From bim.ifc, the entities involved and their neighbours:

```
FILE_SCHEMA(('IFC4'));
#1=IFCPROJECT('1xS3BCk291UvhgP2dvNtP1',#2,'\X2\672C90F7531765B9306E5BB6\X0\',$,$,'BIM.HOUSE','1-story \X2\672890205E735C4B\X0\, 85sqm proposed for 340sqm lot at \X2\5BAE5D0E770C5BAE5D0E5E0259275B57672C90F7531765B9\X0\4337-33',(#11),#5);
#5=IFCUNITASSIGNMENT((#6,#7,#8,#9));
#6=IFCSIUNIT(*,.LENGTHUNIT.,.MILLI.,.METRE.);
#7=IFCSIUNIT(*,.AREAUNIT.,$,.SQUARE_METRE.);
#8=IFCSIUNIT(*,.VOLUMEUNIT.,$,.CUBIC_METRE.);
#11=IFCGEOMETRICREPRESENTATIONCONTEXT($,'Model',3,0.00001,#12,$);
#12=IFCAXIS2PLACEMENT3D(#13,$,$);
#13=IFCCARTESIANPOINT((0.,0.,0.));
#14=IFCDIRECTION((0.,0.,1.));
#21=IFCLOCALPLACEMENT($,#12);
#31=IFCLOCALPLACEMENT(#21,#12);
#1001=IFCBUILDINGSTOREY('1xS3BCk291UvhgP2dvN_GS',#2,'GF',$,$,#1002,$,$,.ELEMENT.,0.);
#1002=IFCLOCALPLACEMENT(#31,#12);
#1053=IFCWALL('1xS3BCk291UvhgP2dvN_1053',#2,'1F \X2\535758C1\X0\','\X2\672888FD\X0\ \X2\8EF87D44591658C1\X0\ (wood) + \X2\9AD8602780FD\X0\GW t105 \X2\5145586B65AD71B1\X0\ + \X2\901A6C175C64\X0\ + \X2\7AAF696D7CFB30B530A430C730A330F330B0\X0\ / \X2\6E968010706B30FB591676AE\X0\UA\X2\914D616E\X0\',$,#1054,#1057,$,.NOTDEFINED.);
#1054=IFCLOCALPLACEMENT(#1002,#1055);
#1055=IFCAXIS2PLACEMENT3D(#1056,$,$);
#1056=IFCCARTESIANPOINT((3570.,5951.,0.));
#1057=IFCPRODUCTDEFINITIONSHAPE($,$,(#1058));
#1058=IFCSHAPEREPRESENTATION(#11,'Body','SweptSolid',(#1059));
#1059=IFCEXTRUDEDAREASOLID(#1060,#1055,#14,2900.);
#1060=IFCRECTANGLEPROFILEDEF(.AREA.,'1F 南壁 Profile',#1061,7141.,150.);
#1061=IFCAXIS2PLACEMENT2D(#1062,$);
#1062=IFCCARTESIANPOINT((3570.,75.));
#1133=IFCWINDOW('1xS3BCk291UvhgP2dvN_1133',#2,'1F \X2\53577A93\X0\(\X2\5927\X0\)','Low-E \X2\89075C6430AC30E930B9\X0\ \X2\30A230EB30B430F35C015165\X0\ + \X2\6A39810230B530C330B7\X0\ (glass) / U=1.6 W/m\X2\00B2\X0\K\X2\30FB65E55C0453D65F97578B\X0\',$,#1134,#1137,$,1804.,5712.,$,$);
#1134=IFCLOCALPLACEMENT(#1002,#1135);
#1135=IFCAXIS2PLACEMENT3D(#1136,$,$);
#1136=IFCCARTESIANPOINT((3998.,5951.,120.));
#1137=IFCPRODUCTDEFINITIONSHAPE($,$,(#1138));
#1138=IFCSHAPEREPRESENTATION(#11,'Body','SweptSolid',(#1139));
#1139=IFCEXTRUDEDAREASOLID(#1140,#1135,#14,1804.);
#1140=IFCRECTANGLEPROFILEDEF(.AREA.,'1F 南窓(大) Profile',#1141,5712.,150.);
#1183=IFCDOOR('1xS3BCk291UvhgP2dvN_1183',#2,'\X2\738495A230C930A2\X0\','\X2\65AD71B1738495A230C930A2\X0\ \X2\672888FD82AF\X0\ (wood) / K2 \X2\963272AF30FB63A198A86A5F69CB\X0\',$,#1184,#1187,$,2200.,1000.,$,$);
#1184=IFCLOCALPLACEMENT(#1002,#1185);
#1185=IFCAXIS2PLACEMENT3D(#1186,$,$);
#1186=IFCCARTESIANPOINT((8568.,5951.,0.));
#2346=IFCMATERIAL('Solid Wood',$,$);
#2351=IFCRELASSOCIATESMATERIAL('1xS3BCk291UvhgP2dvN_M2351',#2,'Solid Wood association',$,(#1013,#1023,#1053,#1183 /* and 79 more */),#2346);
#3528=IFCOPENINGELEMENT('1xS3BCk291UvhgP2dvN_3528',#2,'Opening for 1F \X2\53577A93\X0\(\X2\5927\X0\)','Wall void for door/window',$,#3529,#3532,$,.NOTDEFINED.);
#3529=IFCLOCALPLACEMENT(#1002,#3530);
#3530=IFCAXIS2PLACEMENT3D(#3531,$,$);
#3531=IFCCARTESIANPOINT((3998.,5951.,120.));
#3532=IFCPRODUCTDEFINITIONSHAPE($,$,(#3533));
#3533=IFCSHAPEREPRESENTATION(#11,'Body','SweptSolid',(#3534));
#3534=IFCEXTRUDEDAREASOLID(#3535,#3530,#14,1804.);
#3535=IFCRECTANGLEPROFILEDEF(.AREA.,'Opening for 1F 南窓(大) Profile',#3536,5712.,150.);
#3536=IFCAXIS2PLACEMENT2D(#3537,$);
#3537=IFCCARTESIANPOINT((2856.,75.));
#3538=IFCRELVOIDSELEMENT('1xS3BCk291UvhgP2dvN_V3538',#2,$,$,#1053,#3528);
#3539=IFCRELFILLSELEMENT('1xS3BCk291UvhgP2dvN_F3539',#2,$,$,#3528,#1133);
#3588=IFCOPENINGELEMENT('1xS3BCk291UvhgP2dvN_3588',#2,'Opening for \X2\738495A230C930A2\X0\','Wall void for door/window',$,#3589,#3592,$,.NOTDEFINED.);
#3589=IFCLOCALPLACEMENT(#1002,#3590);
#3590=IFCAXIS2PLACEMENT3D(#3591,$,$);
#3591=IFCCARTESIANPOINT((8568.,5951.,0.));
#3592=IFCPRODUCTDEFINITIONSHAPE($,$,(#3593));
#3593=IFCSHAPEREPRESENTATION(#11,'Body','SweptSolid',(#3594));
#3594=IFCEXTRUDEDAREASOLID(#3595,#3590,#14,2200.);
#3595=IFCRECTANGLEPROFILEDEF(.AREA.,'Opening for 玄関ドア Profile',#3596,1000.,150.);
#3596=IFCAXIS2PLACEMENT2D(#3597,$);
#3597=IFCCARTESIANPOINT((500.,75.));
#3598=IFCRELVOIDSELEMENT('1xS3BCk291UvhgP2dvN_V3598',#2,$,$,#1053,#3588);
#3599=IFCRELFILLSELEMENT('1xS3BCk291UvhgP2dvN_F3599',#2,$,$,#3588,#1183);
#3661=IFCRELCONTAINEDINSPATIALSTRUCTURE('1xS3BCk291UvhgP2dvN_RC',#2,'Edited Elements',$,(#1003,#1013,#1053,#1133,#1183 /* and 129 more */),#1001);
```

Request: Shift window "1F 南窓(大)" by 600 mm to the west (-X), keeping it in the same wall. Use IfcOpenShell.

```python
import ifcopenshell
import ifcopenshell.api.geometry
import ifcopenshell.util.placement

model = ifcopenshell.open("bim.ifc")

window = model.by_guid("1xS3BCk291UvhgP2dvN_1133")
opening = window.FillsVoids[0].RelatingOpeningElement
wall = opening.VoidsElements[0].RelatingBuildingElement

wall_matrix = ifcopenshell.util.placement.get_local_placement(wall.ObjectPlacement)
shift = wall_matrix[:3, 0] * -600.0
before = ifcopenshell.util.placement.get_local_placement(window.ObjectPlacement)[:3, 3].copy()

# The window is not placed relative to its opening, so move both.
for product in (opening, window):
    matrix = ifcopenshell.util.placement.get_local_placement(product.ObjectPlacement)
    matrix[:3, 3] += shift
    ifcopenshell.api.geometry.edit_object_placement(model, product=product, matrix=matrix, is_si=False)

after = ifcopenshell.util.placement.get_local_placement(window.ObjectPlacement)[:3, 3]
print("window moved by", (after - before).round(3) + 0.0)

model.write("bim-out.ifc")
```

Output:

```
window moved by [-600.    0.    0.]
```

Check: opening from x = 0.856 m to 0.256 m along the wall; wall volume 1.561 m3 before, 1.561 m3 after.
